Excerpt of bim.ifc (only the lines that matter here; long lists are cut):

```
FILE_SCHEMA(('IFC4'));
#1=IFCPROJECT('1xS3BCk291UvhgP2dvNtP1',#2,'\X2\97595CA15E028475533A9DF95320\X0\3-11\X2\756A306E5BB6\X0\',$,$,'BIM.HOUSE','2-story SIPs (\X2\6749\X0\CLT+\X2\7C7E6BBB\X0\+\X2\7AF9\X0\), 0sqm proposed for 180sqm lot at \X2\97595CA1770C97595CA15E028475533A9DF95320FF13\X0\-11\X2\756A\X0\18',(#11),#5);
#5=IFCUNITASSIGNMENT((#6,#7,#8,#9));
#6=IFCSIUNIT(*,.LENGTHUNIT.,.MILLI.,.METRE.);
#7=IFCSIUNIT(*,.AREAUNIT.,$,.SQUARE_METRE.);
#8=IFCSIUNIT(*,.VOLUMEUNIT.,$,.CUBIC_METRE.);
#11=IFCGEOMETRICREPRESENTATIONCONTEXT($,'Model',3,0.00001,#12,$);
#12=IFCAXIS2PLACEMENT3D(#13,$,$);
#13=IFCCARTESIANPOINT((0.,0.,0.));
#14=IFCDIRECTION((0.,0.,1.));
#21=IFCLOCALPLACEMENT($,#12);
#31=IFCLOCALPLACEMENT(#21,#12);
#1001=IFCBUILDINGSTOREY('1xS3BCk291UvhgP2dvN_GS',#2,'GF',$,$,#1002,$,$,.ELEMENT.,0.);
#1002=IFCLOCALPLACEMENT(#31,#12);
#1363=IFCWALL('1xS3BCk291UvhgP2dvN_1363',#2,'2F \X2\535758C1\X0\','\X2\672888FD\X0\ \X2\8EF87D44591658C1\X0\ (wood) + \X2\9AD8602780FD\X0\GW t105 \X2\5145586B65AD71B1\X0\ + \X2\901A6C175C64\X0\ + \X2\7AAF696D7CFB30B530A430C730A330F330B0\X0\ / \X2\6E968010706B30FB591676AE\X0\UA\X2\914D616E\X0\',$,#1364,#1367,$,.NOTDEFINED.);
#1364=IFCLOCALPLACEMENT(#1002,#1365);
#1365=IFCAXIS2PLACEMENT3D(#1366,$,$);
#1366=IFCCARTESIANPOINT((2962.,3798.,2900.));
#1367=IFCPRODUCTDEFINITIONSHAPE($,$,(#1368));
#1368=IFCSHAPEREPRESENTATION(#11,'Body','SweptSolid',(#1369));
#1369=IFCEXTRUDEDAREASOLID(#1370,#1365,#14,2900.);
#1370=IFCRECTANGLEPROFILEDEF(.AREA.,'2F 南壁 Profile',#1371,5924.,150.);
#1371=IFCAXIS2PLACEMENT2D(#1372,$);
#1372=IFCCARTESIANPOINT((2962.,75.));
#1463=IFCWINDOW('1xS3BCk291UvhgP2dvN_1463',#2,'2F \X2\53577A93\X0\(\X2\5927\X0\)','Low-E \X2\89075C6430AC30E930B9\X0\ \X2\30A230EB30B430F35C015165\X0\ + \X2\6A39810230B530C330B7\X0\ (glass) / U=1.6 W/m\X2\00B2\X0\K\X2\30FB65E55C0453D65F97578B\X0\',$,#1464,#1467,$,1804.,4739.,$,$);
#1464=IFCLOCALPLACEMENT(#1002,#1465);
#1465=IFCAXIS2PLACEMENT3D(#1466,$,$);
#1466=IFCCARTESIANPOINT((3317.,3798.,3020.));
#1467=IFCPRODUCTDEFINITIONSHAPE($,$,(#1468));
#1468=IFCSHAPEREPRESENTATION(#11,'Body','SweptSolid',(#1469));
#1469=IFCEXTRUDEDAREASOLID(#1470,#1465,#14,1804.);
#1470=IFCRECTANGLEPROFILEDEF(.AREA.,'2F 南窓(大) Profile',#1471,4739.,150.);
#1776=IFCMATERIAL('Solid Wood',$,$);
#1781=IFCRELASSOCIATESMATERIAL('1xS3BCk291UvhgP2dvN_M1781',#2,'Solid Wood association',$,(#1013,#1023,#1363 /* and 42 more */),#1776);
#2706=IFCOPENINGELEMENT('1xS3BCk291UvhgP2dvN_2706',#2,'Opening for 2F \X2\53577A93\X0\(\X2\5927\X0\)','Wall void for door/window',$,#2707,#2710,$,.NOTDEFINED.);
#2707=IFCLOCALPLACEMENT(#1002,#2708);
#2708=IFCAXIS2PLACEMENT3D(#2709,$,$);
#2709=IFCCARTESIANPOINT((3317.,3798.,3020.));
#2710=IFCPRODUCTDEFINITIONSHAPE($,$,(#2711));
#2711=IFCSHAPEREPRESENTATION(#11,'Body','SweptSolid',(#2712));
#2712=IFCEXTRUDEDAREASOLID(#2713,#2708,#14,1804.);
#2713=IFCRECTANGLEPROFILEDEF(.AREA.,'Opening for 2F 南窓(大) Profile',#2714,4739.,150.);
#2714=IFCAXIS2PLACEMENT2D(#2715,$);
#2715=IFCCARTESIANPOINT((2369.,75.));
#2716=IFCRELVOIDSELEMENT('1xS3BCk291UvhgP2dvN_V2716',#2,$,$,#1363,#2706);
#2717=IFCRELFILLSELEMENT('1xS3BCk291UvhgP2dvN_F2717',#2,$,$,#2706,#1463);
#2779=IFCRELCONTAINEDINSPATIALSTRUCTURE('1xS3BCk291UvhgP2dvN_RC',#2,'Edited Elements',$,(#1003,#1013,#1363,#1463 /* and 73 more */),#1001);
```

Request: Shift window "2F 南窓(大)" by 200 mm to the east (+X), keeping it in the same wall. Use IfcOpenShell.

```python
import ifcopenshell
import ifcopenshell.api.geometry
import ifcopenshell.util.placement
import ifcopenshell.util.unit

model = ifcopenshell.open("bim.ifc")
unit_scale = ifcopenshell.util.unit.calculate_unit_scale(model)

window = model.by_guid("1xS3BCk291UvhgP2dvN_1463")
opening = window.FillsVoids[0].RelatingOpeningElement
wall = opening.VoidsElements[0].RelatingBuildingElement

wall_matrix = ifcopenshell.util.placement.get_local_placement(wall.ObjectPlacement)
shift = wall_matrix[:3, 0] * 0.2 / unit_scale
before = ifcopenshell.util.placement.get_local_placement(window.ObjectPlacement)[:3, 3].copy()

# The window is not placed relative to its opening, so move both.
for product in (opening, window):
    matrix = ifcopenshell.util.placement.get_local_placement(product.ObjectPlacement)
    matrix[:3, 3] += shift
    ifcopenshell.api.geometry.edit_object_placement(model, product=product, matrix=matrix, is_si=False)

after = ifcopenshell.util.placement.get_local_placement(window.ObjectPlacement)[:3, 3]
print("window moved by", (after - before).round(3) + 0.0)

model.write("bim-out.ifc")
```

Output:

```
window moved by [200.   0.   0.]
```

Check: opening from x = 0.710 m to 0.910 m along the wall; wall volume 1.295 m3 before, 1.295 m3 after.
